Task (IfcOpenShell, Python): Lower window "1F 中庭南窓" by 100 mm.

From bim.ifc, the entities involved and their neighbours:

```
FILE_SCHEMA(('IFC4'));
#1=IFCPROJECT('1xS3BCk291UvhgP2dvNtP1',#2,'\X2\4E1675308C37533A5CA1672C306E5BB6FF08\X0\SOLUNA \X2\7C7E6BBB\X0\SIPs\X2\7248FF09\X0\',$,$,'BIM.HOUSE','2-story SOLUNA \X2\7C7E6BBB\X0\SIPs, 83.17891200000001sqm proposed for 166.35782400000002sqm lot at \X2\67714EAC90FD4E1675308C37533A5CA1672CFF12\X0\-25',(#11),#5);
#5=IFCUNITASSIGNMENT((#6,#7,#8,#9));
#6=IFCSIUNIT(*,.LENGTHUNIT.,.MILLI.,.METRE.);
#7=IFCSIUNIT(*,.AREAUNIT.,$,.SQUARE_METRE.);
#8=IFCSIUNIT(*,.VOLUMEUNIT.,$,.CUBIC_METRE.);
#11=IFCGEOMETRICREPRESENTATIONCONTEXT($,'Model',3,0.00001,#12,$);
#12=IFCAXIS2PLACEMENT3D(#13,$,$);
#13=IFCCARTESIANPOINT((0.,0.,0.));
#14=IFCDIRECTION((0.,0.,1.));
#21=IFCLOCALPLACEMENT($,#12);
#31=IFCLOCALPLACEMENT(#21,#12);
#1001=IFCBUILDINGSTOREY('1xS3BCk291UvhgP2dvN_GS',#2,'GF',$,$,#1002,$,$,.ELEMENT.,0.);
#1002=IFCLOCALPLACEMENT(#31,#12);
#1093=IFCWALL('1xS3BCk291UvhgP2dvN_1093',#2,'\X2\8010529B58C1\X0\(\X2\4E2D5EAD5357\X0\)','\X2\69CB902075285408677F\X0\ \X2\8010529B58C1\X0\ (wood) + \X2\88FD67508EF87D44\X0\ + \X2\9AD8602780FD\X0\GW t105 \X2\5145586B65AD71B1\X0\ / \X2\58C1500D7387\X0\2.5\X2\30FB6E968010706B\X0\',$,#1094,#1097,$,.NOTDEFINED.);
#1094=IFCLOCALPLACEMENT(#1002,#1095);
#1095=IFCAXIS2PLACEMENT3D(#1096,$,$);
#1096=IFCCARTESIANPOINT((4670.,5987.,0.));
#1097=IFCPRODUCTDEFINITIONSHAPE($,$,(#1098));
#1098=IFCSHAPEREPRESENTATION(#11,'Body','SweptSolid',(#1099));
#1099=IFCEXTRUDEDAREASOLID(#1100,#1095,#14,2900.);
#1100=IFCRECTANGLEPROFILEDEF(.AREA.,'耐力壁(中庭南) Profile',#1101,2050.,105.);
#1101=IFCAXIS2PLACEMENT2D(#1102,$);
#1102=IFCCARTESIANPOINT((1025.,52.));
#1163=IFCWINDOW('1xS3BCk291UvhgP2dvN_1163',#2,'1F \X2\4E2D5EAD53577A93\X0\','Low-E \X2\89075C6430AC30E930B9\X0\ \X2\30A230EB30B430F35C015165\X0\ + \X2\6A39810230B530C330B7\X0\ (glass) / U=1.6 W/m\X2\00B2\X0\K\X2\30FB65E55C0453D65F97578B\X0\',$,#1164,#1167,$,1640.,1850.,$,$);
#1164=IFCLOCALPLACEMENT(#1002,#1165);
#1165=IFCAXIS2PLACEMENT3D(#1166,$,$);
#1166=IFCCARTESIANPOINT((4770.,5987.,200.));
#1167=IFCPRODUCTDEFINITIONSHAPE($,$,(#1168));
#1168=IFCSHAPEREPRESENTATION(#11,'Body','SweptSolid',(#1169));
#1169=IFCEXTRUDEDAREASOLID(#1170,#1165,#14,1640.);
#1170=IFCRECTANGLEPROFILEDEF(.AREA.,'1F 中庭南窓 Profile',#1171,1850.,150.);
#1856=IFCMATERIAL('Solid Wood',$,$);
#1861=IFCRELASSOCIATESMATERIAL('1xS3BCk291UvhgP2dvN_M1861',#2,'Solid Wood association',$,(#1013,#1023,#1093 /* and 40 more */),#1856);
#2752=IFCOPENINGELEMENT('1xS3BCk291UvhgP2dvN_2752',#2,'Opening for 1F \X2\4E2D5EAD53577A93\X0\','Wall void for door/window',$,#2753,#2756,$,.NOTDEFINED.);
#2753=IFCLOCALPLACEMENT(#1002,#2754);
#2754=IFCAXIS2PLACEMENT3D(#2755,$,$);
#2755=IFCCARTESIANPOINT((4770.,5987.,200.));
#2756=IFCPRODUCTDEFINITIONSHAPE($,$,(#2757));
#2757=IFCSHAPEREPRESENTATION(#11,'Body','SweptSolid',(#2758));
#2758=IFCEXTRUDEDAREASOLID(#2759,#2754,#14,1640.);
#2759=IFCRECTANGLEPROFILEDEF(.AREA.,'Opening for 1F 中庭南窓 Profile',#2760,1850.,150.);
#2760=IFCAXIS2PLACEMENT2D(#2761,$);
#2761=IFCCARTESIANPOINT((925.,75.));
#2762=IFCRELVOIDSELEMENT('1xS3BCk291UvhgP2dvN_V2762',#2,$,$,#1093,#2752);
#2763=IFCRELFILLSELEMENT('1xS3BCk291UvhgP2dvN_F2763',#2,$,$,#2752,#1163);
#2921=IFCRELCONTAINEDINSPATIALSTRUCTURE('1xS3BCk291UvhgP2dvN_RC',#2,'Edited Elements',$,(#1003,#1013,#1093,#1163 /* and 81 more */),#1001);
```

```python
import numpy as np
import ifcopenshell
import ifcopenshell.api.geometry
import ifcopenshell.util.placement
import ifcopenshell.util.unit

model = ifcopenshell.open("bim.ifc")
unit_scale = ifcopenshell.util.unit.calculate_unit_scale(model)

window = model.by_guid("1xS3BCk291UvhgP2dvN_1163")
opening = window.FillsVoids[0].RelatingOpeningElement
dz = -0.1 / unit_scale

shift = np.array([0.0, 0.0, dz])
# The window is not placed relative to its opening, so move both.
for product in (opening, window):
    matrix = ifcopenshell.util.placement.get_local_placement(product.ObjectPlacement)
    matrix[:3, 3] += shift
    ifcopenshell.api.geometry.edit_object_placement(model, product=product, matrix=matrix, is_si=False)

print(f"moved by {dz * unit_scale:+.3f} m")

model.write("bim-out.ifc")
```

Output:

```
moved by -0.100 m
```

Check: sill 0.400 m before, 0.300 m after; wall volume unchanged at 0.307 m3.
